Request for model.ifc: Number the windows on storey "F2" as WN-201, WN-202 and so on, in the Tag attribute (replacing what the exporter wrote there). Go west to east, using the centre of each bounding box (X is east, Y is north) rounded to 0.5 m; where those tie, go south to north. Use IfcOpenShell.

First a look at what the model holds.

```python
import ifcopenshell
import ifcopenshell.util.element
import ifcopenshell.util.placement

model = ifcopenshell.open("model.ifc")
print(model.schema)
storey = next(s for s in model.by_type("IfcBuildingStorey") if s.Name == "F2")
windows = [e for e in ifcopenshell.util.element.get_decomposition(storey) if e.is_a("IfcWindow")]
for e in sorted(windows, key=lambda e: e.id()):
    origin = ifcopenshell.util.placement.get_local_placement(e.ObjectPlacement)[:3, 3]
    print(e.id(), e.Tag, e.Name, origin.round(2) + 0.0, sep=" | ")
```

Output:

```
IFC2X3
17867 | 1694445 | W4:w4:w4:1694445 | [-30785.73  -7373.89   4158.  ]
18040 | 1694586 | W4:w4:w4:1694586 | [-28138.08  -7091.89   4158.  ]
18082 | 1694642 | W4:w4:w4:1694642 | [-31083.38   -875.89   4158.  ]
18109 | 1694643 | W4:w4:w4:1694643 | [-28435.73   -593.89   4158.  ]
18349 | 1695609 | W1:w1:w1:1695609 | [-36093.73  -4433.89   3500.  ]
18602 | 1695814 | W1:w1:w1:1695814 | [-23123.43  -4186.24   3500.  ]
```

```python
import ifcopenshell
import ifcopenshell.geom
import ifcopenshell.util.element
import ifcopenshell.util.shape

model = ifcopenshell.open("model.ifc")
settings = ifcopenshell.geom.settings()
settings.set("use-world-coords", True)


def centre(element):
    shape = ifcopenshell.geom.create_shape(settings, element)
    return ifcopenshell.util.shape.get_bbox_centroid(shape.geometry)


storey = next(s for s in model.by_type("IfcBuildingStorey") if s.Name == "F2")
windows = [e for e in ifcopenshell.util.element.get_decomposition(storey) if e.is_a("IfcWindow")]

# Insertion points can sit at a corner or the storey origin, so sort by the geometry (in metres).
centres = {e: centre(e) for e in windows}
windows.sort(key=lambda e: (round(centres[e][0] / 0.5), centres[e][1]))

for i, e in enumerate(windows, start=1):
    number = f"WN-2{i:02d}"
    e.Tag = number
    print(e.id(), number)

model.write("model-out.ifc")
```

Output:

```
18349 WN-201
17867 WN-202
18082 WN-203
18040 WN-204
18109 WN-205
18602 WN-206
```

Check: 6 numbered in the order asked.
